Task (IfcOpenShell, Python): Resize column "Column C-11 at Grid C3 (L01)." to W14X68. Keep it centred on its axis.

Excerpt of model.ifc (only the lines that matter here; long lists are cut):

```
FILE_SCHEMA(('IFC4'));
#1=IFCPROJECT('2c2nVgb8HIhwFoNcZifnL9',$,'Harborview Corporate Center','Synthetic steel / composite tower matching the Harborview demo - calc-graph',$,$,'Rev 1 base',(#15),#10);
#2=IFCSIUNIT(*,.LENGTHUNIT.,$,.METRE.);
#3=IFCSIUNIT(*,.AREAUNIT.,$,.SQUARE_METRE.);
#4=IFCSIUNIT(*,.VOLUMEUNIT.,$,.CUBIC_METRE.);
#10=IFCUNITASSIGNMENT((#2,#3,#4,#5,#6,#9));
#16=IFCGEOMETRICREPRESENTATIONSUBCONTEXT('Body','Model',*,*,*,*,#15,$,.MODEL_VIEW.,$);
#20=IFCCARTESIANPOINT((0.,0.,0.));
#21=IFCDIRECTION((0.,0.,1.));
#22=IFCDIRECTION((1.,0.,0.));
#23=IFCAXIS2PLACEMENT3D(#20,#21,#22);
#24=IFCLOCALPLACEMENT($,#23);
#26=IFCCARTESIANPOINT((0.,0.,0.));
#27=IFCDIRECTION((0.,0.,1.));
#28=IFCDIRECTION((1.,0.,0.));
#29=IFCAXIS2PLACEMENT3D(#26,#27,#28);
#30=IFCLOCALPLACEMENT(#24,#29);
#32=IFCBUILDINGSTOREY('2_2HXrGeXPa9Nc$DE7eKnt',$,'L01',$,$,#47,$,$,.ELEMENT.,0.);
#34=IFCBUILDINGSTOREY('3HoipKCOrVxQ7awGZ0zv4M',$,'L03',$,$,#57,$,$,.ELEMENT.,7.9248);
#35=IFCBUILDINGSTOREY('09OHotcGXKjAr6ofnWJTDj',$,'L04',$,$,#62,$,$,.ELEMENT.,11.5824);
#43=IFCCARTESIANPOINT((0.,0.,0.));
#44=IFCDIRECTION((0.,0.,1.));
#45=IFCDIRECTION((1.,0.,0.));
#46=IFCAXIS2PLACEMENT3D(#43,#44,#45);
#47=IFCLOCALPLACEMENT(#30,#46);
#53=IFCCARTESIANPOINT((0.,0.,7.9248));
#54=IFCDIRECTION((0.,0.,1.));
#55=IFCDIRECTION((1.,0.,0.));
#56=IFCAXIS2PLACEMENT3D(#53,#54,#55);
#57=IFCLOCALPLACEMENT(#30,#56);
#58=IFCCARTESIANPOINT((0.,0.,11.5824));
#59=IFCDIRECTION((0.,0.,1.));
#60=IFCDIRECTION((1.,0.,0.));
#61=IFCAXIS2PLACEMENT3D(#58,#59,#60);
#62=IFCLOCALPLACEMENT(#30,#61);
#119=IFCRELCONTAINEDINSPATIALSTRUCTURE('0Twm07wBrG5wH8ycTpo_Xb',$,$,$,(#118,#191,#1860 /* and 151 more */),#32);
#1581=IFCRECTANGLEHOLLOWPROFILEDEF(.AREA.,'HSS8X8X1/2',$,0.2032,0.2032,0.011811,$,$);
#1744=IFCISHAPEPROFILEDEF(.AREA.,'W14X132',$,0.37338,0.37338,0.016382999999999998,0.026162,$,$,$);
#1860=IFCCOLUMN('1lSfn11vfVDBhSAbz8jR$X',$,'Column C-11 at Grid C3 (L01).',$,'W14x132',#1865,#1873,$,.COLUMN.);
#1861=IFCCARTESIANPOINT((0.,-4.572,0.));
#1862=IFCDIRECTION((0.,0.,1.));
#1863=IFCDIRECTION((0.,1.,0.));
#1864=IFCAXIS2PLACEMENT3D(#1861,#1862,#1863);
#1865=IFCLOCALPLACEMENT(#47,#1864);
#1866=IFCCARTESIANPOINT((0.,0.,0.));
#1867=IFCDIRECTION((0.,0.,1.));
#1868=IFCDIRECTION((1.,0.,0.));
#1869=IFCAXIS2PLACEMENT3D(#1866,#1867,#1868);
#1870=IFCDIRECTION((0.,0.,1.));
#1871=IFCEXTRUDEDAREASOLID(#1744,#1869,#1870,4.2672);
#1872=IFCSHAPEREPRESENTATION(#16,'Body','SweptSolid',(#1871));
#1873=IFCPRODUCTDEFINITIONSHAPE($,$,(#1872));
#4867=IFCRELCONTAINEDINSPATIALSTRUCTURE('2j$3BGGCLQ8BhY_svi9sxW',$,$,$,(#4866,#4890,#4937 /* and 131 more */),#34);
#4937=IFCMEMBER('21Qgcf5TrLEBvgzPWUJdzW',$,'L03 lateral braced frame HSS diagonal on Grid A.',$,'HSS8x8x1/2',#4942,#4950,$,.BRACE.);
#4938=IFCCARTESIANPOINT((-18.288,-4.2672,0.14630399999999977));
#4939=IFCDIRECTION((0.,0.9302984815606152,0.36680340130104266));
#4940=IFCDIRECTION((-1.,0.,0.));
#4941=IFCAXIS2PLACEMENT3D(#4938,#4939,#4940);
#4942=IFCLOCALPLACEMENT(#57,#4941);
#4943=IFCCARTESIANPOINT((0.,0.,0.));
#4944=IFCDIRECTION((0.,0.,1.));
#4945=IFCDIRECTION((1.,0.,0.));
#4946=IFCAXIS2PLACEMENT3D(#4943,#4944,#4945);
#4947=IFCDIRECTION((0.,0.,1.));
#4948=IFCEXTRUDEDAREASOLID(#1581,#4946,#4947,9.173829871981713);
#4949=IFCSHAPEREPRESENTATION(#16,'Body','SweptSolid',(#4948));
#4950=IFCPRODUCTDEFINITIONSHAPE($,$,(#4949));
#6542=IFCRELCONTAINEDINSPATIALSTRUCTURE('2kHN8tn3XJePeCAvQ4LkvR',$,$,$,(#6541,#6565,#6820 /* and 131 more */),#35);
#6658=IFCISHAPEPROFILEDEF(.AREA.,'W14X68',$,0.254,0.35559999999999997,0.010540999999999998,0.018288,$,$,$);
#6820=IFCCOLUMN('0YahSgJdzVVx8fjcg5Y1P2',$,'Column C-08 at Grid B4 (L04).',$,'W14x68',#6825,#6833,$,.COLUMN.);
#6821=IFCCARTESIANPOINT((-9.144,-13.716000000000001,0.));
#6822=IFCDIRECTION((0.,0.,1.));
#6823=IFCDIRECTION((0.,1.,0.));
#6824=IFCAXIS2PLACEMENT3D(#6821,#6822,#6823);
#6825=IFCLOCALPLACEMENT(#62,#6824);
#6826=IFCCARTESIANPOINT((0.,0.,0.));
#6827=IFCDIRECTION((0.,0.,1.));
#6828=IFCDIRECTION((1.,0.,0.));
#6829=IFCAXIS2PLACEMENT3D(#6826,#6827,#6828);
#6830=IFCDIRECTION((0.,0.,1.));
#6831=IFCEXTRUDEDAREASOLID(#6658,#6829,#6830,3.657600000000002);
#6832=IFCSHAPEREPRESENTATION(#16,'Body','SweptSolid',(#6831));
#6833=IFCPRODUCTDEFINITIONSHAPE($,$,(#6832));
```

```python
import ifcopenshell
import ifcopenshell.util.element
import ifcopenshell.util.representation

model = ifcopenshell.open("model.ifc")

member = model.by_guid("1lSfn11vfVDBhSAbz8jR$X")
source = next(p for p in model.by_type("IfcIShapeProfileDef") if p.ProfileName == "W14X68")

body = ifcopenshell.util.representation.get_representation(member, "Model", "Body")
solid = body.Items[0]
old_profile = solid.SweptArea

# Copy the section's sizes but keep this member's own profile position.
profile = ifcopenshell.util.element.copy(model, source)
profile.Position = old_profile.Position
solid.SweptArea = profile
if not model.get_total_inverses(old_profile):
    ifcopenshell.util.element.remove_deep2(model, old_profile)

print(solid.SweptArea)

model.write("model_v2.ifc")
```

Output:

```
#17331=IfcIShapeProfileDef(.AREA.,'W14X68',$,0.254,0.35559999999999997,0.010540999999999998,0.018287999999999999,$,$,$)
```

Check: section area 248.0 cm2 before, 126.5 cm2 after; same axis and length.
